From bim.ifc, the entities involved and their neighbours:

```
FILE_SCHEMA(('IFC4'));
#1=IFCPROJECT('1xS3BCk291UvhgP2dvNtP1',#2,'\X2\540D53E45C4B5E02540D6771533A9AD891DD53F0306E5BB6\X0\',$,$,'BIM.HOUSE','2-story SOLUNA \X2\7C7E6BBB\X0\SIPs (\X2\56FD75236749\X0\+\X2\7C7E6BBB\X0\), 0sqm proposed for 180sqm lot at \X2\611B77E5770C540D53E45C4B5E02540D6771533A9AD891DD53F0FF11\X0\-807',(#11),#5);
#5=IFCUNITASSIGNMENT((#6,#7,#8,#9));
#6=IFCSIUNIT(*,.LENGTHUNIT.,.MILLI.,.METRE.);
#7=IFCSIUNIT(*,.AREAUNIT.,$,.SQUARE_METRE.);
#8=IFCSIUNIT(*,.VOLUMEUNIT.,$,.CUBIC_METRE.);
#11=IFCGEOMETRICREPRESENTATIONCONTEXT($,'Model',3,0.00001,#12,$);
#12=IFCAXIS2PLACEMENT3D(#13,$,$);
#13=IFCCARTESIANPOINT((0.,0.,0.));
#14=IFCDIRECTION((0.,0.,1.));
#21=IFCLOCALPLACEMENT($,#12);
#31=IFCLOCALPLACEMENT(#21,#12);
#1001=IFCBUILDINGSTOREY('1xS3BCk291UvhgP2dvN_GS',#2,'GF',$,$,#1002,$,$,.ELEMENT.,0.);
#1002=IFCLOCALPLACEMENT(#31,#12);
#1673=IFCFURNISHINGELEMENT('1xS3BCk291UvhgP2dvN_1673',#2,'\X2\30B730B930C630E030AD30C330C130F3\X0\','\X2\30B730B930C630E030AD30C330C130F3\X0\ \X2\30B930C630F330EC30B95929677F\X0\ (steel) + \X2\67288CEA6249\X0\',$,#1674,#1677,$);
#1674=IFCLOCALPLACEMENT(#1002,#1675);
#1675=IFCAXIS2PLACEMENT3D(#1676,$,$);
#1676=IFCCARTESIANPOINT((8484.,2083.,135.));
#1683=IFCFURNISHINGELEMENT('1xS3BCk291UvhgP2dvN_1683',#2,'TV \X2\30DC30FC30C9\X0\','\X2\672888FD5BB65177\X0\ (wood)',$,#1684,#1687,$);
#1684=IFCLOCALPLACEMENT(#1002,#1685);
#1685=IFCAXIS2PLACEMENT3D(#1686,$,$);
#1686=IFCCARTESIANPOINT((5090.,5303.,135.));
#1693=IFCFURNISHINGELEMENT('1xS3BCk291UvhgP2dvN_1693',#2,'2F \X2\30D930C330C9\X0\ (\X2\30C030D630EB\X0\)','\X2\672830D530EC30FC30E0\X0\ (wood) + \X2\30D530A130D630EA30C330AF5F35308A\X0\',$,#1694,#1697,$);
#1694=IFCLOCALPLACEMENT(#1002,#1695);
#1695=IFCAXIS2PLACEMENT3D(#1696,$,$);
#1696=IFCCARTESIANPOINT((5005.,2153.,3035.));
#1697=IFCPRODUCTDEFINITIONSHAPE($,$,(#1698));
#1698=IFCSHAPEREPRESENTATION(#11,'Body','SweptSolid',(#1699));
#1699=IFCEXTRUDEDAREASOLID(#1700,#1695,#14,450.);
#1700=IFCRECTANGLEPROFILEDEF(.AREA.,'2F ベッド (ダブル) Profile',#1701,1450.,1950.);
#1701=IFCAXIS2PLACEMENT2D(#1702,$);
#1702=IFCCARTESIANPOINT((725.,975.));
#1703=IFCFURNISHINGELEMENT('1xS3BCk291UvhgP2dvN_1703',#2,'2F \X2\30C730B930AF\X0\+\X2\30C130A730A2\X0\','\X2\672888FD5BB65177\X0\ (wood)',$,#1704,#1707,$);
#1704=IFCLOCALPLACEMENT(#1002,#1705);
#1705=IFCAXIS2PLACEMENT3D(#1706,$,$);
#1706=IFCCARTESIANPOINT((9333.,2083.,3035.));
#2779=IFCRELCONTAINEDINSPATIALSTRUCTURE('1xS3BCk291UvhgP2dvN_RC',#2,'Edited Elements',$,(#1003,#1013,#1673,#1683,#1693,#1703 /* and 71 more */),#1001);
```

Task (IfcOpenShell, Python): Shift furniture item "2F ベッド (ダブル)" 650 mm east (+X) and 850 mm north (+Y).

```python
import ifcopenshell
import ifcopenshell.api.geometry
import ifcopenshell.util.placement

model = ifcopenshell.open("bim.ifc")

item = model.by_id(1693)
matrix = ifcopenshell.util.placement.get_local_placement(item.ObjectPlacement)
matrix[0, 3] += 650.0
matrix[1, 3] += 850.0
ifcopenshell.api.geometry.edit_object_placement(model, product=item, matrix=matrix, is_si=False)

print(ifcopenshell.util.placement.get_local_placement(item.ObjectPlacement).round(3) + 0.0)

model.write("bim_updated.ifc")
```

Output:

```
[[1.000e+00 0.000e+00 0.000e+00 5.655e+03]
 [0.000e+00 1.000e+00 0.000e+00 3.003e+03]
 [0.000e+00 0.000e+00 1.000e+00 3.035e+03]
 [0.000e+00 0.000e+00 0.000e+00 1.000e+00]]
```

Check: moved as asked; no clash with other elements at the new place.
